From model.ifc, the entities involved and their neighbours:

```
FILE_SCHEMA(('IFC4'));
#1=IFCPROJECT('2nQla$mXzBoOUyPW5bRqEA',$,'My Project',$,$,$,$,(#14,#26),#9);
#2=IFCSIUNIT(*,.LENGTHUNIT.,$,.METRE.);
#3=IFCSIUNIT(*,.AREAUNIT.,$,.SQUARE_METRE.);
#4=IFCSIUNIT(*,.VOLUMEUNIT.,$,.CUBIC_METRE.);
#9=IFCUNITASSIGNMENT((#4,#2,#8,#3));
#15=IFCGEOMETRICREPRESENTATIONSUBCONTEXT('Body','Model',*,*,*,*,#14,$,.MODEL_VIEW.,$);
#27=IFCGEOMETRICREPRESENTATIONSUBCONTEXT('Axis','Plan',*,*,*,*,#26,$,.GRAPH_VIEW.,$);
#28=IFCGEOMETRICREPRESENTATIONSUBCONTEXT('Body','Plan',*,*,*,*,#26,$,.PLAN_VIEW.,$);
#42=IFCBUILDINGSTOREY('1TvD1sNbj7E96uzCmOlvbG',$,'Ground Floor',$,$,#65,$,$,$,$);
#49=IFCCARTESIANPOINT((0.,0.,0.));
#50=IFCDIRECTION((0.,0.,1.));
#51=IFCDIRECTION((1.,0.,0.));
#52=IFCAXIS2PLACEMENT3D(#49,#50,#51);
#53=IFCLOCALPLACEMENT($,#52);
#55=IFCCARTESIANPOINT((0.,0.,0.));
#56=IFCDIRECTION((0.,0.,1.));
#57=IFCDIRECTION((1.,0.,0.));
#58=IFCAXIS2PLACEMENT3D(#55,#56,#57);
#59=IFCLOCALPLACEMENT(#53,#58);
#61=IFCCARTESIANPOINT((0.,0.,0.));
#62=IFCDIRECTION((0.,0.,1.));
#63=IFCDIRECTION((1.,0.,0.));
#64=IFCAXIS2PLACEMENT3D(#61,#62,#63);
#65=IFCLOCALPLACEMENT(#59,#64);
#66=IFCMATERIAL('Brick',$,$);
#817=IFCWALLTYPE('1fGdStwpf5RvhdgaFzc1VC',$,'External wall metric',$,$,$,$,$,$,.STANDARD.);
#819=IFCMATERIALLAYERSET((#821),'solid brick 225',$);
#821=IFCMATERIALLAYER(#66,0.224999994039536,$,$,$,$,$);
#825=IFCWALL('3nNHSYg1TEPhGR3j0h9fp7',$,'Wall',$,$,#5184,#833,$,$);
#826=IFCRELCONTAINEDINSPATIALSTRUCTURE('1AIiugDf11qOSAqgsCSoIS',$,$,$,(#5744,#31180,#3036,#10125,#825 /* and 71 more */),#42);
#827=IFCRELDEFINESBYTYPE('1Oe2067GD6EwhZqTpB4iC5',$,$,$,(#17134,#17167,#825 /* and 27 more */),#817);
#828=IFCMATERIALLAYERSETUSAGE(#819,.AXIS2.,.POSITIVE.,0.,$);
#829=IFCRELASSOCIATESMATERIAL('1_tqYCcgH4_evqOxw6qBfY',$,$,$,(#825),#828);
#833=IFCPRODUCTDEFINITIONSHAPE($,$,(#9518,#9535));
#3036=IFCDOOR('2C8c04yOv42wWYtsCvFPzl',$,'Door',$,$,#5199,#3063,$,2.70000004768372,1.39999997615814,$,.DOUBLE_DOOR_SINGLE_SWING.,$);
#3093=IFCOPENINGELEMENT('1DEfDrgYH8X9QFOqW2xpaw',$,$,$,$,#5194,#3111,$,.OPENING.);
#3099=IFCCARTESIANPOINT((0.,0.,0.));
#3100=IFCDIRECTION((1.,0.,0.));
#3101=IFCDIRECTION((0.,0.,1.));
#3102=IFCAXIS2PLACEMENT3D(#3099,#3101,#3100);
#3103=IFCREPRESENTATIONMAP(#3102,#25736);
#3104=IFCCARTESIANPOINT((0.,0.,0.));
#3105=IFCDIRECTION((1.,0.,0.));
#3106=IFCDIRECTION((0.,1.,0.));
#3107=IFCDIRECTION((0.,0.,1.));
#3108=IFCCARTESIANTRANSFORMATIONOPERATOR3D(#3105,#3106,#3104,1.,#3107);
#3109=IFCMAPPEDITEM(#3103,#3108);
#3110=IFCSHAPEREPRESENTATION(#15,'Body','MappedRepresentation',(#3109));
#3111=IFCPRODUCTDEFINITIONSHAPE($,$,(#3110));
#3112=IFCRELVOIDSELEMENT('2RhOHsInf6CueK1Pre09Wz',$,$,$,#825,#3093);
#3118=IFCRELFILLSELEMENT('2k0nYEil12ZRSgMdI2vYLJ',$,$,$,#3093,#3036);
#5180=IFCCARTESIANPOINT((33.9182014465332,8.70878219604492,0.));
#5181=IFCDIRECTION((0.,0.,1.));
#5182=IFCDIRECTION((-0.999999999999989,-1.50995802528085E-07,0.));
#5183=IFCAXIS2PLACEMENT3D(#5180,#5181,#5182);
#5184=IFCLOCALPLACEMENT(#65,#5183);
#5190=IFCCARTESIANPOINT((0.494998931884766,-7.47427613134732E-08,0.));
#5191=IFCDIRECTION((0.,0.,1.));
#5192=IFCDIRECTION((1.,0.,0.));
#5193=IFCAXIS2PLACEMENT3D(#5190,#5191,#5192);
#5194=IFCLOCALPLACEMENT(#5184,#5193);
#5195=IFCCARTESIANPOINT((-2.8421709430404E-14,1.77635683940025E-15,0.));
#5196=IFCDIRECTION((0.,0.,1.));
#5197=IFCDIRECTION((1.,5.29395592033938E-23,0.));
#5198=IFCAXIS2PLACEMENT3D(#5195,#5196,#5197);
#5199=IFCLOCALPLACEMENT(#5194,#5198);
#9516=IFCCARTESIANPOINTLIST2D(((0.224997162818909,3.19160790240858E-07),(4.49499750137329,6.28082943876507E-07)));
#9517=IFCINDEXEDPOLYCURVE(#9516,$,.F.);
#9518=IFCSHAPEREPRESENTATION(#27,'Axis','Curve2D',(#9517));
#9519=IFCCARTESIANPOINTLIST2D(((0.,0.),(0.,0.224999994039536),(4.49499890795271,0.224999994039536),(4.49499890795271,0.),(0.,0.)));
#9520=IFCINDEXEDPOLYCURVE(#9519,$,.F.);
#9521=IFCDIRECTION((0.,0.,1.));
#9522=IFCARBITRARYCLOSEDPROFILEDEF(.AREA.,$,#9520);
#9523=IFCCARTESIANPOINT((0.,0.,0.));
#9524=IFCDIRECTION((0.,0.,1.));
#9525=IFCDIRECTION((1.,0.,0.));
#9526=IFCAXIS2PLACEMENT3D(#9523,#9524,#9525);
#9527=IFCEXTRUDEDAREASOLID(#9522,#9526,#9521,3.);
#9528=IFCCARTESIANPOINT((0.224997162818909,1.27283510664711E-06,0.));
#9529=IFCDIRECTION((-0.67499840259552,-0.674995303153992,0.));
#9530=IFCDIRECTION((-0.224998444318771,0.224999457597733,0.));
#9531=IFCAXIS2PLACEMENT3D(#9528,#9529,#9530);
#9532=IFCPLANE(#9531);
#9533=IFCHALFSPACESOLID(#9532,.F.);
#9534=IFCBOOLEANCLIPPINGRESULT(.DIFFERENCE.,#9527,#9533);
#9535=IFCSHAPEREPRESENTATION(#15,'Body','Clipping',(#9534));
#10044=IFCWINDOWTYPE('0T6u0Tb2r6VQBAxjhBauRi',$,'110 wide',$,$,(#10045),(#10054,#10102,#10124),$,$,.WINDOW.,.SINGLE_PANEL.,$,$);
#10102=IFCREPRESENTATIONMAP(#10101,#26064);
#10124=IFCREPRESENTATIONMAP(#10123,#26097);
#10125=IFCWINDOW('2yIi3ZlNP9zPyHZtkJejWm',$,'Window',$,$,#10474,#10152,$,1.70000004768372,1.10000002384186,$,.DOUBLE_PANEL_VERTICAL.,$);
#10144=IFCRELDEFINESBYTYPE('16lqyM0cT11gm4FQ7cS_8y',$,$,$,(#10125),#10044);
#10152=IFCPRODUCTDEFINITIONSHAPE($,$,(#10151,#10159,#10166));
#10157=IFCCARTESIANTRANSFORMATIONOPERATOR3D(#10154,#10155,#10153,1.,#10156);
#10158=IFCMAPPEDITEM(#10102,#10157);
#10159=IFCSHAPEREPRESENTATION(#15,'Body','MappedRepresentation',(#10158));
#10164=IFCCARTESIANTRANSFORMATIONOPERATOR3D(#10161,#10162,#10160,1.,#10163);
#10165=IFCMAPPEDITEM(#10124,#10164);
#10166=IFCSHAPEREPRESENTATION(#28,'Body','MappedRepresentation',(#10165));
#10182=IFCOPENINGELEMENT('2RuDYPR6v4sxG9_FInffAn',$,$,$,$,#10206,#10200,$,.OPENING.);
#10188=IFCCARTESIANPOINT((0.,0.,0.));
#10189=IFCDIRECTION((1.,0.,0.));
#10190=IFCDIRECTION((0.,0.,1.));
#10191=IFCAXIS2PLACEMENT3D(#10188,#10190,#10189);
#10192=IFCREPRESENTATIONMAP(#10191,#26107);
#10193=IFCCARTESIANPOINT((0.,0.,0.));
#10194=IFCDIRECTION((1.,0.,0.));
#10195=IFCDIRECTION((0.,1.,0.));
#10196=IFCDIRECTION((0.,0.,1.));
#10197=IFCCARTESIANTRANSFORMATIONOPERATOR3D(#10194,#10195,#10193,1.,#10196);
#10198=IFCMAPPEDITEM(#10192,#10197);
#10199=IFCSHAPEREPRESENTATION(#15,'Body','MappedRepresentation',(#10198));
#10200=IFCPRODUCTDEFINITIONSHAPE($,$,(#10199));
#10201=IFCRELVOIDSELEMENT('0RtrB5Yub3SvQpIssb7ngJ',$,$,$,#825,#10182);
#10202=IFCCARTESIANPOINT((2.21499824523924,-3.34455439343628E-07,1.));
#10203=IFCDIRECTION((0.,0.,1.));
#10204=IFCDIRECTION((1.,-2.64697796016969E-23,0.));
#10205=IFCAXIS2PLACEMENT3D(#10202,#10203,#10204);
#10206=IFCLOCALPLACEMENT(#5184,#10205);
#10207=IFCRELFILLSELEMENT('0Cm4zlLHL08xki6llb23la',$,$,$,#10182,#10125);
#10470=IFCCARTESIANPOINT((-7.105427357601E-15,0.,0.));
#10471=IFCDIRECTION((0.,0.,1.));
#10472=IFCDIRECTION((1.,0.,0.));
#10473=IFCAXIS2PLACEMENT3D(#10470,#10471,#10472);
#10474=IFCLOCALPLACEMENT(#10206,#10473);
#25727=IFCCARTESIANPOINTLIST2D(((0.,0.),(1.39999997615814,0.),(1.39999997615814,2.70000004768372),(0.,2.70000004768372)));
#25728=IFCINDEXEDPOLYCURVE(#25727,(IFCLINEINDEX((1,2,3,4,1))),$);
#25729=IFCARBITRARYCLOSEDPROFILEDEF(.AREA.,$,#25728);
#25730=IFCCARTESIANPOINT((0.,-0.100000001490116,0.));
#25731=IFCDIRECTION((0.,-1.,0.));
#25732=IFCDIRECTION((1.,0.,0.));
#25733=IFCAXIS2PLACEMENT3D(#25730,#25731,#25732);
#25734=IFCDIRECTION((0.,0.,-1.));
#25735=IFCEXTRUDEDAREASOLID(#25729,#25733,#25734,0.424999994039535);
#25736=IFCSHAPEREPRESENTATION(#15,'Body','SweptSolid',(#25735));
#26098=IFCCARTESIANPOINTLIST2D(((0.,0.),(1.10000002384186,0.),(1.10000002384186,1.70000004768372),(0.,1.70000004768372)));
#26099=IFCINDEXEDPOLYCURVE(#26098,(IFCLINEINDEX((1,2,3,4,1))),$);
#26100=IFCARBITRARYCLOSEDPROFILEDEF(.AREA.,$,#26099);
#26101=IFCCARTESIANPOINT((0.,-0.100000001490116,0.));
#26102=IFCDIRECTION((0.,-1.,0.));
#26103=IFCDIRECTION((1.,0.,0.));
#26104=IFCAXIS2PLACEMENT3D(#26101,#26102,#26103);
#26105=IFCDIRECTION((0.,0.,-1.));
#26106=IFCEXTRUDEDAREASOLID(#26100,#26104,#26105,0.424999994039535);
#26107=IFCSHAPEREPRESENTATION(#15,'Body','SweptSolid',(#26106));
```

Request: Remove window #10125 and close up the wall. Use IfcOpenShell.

```python
import ifcopenshell
import ifcopenshell.api.feature
import ifcopenshell.api.root
import ifcopenshell.geom
import ifcopenshell.util.shape

model = ifcopenshell.open("model.ifc")
settings = ifcopenshell.geom.settings()


def volume(element):
    """Net volume in cubic metres, openings subtracted."""
    shape = ifcopenshell.geom.create_shape(settings, element)
    return ifcopenshell.util.shape.get_volume(shape.geometry)


window = model.by_id(10125)
opening = window.FillsVoids[0].RelatingOpeningElement
wall = opening.VoidsElements[0].RelatingBuildingElement
before = volume(wall)

ifcopenshell.api.root.remove_product(model, product=window)
ifcopenshell.api.feature.remove_feature(model, feature=opening)

after = volume(wall)

print(f"wall volume {before:.3f} -> {after:.3f} m3")

model.write("model-out.ifc")
```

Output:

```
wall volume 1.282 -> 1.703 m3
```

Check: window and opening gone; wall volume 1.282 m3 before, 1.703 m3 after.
